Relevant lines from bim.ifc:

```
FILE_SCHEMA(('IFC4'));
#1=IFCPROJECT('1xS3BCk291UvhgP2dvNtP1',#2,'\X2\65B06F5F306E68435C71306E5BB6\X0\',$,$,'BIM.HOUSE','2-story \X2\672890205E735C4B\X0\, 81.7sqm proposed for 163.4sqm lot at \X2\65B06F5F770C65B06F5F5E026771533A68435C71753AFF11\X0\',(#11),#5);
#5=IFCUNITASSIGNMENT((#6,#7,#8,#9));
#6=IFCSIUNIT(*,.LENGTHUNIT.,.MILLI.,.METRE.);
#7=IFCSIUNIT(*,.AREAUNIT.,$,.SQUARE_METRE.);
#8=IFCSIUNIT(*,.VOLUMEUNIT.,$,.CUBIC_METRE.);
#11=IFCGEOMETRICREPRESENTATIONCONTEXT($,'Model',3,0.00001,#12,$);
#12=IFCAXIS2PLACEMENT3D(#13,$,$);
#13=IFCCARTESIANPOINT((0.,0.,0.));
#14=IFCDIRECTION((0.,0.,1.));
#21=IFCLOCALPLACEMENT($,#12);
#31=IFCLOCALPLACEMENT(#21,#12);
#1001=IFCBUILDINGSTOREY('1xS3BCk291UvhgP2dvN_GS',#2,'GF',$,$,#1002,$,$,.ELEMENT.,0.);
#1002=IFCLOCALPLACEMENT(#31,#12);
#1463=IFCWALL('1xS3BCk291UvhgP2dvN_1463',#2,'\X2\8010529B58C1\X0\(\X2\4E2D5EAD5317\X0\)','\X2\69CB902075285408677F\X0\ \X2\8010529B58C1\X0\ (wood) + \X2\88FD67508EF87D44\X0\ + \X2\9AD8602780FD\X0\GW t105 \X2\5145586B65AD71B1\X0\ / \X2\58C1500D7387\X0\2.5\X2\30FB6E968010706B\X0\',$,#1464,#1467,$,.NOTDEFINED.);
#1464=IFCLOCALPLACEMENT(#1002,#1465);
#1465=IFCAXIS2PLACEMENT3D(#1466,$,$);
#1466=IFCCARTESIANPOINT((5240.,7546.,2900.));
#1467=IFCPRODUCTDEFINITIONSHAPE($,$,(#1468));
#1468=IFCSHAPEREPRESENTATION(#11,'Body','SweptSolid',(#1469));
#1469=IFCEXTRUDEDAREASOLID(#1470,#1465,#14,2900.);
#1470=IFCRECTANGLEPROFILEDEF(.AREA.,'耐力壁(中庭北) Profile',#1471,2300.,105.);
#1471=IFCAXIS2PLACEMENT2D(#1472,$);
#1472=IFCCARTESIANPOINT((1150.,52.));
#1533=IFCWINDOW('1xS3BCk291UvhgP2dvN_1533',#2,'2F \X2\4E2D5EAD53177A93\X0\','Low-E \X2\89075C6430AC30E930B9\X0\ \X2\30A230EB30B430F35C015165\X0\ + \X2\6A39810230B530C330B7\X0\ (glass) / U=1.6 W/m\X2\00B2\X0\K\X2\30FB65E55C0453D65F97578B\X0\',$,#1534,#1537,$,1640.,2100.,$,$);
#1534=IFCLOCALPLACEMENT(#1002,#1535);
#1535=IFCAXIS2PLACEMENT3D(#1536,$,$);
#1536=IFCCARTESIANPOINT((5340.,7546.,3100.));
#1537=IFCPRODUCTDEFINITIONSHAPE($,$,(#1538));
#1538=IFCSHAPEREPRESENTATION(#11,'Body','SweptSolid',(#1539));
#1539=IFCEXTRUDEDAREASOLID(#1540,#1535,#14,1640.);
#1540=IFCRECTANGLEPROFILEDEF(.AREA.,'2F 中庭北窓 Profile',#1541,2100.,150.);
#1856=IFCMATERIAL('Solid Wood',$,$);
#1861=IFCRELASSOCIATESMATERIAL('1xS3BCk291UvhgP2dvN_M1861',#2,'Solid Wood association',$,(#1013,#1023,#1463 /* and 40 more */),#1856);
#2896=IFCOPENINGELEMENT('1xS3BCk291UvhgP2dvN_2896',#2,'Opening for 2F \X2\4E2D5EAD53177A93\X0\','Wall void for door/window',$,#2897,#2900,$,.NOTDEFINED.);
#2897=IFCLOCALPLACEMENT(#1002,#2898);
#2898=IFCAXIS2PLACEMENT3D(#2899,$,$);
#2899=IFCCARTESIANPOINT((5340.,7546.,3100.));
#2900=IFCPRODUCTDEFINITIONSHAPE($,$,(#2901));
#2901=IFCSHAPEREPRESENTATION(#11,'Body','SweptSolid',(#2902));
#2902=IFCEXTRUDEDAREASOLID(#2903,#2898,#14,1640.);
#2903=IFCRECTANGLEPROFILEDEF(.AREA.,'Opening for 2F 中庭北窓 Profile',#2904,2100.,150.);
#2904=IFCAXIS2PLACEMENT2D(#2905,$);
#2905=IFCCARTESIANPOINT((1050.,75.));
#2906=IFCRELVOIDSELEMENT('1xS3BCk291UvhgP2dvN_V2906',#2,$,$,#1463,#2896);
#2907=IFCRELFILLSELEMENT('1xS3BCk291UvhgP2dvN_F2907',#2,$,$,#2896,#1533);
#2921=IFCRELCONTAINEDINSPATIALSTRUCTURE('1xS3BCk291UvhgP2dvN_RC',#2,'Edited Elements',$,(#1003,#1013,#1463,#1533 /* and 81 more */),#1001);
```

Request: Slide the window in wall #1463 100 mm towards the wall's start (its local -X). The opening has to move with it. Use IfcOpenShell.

```python
import ifcopenshell
import ifcopenshell.api.geometry
import ifcopenshell.util.placement
import ifcopenshell.util.unit

model = ifcopenshell.open("bim.ifc")
unit_scale = ifcopenshell.util.unit.calculate_unit_scale(model)

window = model.by_id(1533)
opening = window.FillsVoids[0].RelatingOpeningElement
wall = opening.VoidsElements[0].RelatingBuildingElement

wall_matrix = ifcopenshell.util.placement.get_local_placement(wall.ObjectPlacement)
shift = wall_matrix[:3, 0] * -0.1 / unit_scale
before = ifcopenshell.util.placement.get_local_placement(window.ObjectPlacement)[:3, 3].copy()

# The window is not placed relative to its opening, so move both.
for product in (opening, window):
    matrix = ifcopenshell.util.placement.get_local_placement(product.ObjectPlacement)
    matrix[:3, 3] += shift
    ifcopenshell.api.geometry.edit_object_placement(model, product=product, matrix=matrix, is_si=False)

after = ifcopenshell.util.placement.get_local_placement(window.ObjectPlacement)[:3, 3]
print("window moved by", (after - before).round(3) + 0.0)

model.write("bim_v2.ifc")
```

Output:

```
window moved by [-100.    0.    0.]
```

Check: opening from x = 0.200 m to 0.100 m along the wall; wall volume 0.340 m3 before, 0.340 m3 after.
